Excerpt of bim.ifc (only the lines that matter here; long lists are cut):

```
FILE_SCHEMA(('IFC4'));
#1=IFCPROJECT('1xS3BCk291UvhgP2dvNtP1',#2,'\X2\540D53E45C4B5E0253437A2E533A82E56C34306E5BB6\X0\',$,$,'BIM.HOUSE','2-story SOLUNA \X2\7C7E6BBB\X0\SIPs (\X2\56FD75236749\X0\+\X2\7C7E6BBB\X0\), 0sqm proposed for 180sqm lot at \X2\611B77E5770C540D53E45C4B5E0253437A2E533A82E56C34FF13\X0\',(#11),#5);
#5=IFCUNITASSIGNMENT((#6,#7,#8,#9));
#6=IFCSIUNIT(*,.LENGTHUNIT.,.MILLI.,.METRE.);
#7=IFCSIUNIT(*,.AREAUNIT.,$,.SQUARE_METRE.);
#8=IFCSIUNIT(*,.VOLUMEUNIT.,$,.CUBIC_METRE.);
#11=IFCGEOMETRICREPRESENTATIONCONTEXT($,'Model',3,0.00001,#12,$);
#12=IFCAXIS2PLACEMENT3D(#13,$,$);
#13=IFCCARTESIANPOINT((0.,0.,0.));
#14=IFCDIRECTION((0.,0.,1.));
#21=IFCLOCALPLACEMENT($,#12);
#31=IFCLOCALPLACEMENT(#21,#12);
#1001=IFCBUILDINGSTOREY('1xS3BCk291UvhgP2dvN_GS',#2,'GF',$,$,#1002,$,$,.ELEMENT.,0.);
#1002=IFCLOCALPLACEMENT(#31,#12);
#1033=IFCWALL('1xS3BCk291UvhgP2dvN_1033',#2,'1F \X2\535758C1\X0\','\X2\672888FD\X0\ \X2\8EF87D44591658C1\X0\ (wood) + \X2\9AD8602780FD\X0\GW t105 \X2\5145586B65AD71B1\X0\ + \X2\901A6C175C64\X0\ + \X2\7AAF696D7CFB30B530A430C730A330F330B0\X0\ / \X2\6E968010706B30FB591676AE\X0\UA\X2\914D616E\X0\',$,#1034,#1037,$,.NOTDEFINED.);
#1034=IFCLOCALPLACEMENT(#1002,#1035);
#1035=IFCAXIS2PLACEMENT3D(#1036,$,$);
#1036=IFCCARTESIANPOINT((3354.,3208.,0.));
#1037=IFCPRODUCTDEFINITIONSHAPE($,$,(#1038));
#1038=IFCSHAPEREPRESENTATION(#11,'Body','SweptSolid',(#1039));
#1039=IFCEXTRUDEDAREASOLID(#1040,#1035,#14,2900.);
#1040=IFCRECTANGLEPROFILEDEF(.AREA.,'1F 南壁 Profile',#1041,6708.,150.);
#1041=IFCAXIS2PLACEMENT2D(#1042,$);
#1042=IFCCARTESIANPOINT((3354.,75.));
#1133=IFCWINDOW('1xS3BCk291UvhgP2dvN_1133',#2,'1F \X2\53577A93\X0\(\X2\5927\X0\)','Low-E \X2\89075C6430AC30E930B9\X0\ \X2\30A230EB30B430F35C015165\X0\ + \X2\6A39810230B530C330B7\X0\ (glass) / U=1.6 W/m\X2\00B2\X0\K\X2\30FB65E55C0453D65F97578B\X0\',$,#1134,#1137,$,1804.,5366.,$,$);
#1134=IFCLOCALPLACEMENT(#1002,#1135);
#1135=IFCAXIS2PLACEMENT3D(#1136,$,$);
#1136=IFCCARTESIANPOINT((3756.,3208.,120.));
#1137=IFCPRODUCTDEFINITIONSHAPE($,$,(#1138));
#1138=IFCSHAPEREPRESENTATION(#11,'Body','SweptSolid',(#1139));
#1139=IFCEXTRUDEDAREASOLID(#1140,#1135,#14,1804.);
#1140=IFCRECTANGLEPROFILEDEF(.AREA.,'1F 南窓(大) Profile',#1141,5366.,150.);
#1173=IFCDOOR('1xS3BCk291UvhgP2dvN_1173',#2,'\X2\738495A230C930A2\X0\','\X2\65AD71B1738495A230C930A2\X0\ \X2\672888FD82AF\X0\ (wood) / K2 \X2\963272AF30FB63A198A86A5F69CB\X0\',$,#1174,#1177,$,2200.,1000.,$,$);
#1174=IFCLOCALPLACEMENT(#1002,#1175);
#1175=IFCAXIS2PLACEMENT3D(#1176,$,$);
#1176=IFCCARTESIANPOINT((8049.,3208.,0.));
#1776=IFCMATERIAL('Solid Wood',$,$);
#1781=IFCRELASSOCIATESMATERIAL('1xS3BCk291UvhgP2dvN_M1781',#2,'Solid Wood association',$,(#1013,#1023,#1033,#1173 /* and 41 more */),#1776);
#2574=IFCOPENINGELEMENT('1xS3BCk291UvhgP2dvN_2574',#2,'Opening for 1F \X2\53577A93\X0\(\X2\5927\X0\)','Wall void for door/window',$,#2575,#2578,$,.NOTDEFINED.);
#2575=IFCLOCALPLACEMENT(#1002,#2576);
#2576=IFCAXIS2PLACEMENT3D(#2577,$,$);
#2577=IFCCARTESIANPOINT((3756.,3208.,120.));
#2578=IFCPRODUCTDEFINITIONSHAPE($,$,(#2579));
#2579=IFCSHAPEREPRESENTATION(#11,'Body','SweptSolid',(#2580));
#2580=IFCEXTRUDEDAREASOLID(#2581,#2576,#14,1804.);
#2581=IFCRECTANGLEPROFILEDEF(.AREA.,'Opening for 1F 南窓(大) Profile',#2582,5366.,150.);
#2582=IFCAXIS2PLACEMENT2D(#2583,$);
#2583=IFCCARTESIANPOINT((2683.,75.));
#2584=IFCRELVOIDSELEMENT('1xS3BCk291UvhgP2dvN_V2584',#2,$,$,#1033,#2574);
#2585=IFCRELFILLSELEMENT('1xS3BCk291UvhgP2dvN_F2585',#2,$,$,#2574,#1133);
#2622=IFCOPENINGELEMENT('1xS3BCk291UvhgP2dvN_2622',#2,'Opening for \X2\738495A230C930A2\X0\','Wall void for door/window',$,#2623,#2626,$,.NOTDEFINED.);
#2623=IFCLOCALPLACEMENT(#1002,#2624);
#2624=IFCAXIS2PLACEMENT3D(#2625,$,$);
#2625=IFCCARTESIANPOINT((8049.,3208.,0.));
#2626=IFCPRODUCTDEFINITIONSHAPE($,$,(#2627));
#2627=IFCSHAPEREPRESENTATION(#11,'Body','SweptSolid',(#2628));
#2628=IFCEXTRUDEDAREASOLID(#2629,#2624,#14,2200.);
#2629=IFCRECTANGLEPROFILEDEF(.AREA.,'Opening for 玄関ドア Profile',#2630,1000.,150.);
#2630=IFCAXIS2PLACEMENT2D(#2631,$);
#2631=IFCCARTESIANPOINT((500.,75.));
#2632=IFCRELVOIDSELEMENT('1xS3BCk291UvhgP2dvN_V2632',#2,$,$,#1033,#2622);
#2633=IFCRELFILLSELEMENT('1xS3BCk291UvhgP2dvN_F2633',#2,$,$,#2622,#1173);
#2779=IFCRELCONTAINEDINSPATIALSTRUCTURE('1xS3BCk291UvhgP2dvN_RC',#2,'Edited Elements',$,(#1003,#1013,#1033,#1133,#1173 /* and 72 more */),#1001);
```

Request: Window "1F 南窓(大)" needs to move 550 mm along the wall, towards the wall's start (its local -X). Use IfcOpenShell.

```python
import ifcopenshell
import ifcopenshell.api.geometry
import ifcopenshell.util.placement

model = ifcopenshell.open("bim.ifc")

window = model.by_guid("1xS3BCk291UvhgP2dvN_1133")
opening = window.FillsVoids[0].RelatingOpeningElement
wall = opening.VoidsElements[0].RelatingBuildingElement

wall_matrix = ifcopenshell.util.placement.get_local_placement(wall.ObjectPlacement)
shift = wall_matrix[:3, 0] * -550.0
before = ifcopenshell.util.placement.get_local_placement(window.ObjectPlacement)[:3, 3].copy()

# The window is not placed relative to its opening, so move both.
for product in (opening, window):
    matrix = ifcopenshell.util.placement.get_local_placement(product.ObjectPlacement)
    matrix[:3, 3] += shift
    ifcopenshell.api.geometry.edit_object_placement(model, product=product, matrix=matrix, is_si=False)

after = ifcopenshell.util.placement.get_local_placement(window.ObjectPlacement)[:3, 3]
print("window moved by", (after - before).round(3) + 0.0)

model.write("bim_updated.ifc")
```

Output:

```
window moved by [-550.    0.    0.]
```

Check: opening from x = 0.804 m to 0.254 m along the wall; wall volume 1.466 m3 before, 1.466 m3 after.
